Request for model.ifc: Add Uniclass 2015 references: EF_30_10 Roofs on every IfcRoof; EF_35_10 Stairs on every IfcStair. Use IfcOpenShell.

First a look at what the model holds.

```python
import ifcopenshell

model = ifcopenshell.open("model.ifc")
print(model.schema)
print("classifications:", [c.Name for c in model.by_type("IfcClassification")])
for ifc_class in ("IfcDoor", "IfcRoof", "IfcStair", "IfcWall", "IfcWindow"):
    print(ifc_class, len(model.by_type(ifc_class)))
```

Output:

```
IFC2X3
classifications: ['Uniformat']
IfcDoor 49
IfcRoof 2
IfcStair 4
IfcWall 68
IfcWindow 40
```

```python
import ifcopenshell
import ifcopenshell.api.classification

model = ifcopenshell.open("model.ifc")

# IFC2X3 requires Source and Edition and has no link from the project to the system.
system = model.create_entity("IfcClassification", Source="NBS", Edition="2015", Name="Uniclass 2015")

codes = {
    "IfcRoof": ("EF_30_10", "Roofs"),
    "IfcStair": ("EF_35_10", "Stairs"),
}
for ifc_class, (code, name) in codes.items():
    products = model.by_type(ifc_class)
    ifcopenshell.api.classification.add_reference(
        model, products=products, classification=system, identification=code, name=name
    )
    print(code, len(products))

model.write("model_edited.ifc")
```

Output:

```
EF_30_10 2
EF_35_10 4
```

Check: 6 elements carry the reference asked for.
